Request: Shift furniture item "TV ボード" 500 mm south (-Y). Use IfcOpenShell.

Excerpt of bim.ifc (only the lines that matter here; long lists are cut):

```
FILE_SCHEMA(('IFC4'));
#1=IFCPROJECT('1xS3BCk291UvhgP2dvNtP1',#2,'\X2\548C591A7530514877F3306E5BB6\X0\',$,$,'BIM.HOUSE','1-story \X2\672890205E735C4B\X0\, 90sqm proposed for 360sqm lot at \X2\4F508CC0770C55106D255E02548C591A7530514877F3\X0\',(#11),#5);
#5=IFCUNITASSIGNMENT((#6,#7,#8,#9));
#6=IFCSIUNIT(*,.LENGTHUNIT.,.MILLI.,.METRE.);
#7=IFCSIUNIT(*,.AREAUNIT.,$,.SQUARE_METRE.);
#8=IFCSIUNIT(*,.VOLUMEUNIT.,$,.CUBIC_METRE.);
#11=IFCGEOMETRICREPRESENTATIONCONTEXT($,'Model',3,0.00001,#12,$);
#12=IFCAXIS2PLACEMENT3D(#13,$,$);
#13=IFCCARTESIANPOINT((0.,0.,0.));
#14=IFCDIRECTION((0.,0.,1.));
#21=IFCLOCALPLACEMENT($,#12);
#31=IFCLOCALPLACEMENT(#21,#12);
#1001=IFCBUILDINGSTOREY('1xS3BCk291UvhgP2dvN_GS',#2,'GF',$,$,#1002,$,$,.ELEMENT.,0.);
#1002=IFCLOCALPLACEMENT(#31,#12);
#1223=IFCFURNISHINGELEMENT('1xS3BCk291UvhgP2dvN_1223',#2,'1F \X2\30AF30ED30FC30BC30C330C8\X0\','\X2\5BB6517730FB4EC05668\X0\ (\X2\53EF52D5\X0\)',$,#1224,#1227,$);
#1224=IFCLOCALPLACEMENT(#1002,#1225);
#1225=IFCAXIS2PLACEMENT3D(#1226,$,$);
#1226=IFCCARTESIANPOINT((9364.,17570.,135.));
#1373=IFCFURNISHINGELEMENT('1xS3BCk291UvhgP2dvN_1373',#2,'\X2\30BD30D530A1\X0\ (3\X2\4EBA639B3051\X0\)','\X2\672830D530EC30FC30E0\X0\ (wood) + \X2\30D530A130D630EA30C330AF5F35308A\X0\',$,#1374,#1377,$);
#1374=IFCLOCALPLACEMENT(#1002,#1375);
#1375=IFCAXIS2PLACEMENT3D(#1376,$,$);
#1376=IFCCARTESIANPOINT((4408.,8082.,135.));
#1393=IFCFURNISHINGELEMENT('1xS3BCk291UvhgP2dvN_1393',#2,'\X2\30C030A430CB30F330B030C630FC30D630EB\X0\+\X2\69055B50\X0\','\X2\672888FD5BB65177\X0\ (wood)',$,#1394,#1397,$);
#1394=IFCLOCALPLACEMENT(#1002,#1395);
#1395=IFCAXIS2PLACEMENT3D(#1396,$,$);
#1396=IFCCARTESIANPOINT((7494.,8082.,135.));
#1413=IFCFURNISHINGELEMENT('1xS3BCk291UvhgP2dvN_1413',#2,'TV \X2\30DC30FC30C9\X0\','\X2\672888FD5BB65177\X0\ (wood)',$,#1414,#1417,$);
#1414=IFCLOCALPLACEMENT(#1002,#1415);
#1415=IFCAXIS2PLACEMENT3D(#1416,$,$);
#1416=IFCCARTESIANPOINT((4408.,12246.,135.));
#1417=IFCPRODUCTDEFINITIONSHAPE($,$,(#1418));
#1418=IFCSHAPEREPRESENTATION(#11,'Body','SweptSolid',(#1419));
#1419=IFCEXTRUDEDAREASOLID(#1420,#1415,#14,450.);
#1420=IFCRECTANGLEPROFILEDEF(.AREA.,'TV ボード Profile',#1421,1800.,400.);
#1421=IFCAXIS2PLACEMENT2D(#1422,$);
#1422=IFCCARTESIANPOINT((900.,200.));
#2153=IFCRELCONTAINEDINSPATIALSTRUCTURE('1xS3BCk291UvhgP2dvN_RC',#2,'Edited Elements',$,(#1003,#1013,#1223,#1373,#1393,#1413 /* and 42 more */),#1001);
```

```python
import ifcopenshell
import ifcopenshell.api.geometry
import ifcopenshell.util.placement
import ifcopenshell.util.unit

model = ifcopenshell.open("bim.ifc")
unit_scale = ifcopenshell.util.unit.calculate_unit_scale(model)

item = model.by_guid("1xS3BCk291UvhgP2dvN_1413")
matrix = ifcopenshell.util.placement.get_local_placement(item.ObjectPlacement)
matrix[1, 3] -= 0.5 / unit_scale
ifcopenshell.api.geometry.edit_object_placement(model, product=item, matrix=matrix, is_si=False)

print(ifcopenshell.util.placement.get_local_placement(item.ObjectPlacement).round(3) + 0.0)

model.write("bim_edited.ifc")
```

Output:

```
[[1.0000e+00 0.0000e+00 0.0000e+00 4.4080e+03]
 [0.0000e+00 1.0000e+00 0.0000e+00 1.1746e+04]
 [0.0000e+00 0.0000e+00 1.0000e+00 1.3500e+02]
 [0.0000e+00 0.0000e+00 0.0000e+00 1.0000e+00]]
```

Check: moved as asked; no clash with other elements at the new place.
